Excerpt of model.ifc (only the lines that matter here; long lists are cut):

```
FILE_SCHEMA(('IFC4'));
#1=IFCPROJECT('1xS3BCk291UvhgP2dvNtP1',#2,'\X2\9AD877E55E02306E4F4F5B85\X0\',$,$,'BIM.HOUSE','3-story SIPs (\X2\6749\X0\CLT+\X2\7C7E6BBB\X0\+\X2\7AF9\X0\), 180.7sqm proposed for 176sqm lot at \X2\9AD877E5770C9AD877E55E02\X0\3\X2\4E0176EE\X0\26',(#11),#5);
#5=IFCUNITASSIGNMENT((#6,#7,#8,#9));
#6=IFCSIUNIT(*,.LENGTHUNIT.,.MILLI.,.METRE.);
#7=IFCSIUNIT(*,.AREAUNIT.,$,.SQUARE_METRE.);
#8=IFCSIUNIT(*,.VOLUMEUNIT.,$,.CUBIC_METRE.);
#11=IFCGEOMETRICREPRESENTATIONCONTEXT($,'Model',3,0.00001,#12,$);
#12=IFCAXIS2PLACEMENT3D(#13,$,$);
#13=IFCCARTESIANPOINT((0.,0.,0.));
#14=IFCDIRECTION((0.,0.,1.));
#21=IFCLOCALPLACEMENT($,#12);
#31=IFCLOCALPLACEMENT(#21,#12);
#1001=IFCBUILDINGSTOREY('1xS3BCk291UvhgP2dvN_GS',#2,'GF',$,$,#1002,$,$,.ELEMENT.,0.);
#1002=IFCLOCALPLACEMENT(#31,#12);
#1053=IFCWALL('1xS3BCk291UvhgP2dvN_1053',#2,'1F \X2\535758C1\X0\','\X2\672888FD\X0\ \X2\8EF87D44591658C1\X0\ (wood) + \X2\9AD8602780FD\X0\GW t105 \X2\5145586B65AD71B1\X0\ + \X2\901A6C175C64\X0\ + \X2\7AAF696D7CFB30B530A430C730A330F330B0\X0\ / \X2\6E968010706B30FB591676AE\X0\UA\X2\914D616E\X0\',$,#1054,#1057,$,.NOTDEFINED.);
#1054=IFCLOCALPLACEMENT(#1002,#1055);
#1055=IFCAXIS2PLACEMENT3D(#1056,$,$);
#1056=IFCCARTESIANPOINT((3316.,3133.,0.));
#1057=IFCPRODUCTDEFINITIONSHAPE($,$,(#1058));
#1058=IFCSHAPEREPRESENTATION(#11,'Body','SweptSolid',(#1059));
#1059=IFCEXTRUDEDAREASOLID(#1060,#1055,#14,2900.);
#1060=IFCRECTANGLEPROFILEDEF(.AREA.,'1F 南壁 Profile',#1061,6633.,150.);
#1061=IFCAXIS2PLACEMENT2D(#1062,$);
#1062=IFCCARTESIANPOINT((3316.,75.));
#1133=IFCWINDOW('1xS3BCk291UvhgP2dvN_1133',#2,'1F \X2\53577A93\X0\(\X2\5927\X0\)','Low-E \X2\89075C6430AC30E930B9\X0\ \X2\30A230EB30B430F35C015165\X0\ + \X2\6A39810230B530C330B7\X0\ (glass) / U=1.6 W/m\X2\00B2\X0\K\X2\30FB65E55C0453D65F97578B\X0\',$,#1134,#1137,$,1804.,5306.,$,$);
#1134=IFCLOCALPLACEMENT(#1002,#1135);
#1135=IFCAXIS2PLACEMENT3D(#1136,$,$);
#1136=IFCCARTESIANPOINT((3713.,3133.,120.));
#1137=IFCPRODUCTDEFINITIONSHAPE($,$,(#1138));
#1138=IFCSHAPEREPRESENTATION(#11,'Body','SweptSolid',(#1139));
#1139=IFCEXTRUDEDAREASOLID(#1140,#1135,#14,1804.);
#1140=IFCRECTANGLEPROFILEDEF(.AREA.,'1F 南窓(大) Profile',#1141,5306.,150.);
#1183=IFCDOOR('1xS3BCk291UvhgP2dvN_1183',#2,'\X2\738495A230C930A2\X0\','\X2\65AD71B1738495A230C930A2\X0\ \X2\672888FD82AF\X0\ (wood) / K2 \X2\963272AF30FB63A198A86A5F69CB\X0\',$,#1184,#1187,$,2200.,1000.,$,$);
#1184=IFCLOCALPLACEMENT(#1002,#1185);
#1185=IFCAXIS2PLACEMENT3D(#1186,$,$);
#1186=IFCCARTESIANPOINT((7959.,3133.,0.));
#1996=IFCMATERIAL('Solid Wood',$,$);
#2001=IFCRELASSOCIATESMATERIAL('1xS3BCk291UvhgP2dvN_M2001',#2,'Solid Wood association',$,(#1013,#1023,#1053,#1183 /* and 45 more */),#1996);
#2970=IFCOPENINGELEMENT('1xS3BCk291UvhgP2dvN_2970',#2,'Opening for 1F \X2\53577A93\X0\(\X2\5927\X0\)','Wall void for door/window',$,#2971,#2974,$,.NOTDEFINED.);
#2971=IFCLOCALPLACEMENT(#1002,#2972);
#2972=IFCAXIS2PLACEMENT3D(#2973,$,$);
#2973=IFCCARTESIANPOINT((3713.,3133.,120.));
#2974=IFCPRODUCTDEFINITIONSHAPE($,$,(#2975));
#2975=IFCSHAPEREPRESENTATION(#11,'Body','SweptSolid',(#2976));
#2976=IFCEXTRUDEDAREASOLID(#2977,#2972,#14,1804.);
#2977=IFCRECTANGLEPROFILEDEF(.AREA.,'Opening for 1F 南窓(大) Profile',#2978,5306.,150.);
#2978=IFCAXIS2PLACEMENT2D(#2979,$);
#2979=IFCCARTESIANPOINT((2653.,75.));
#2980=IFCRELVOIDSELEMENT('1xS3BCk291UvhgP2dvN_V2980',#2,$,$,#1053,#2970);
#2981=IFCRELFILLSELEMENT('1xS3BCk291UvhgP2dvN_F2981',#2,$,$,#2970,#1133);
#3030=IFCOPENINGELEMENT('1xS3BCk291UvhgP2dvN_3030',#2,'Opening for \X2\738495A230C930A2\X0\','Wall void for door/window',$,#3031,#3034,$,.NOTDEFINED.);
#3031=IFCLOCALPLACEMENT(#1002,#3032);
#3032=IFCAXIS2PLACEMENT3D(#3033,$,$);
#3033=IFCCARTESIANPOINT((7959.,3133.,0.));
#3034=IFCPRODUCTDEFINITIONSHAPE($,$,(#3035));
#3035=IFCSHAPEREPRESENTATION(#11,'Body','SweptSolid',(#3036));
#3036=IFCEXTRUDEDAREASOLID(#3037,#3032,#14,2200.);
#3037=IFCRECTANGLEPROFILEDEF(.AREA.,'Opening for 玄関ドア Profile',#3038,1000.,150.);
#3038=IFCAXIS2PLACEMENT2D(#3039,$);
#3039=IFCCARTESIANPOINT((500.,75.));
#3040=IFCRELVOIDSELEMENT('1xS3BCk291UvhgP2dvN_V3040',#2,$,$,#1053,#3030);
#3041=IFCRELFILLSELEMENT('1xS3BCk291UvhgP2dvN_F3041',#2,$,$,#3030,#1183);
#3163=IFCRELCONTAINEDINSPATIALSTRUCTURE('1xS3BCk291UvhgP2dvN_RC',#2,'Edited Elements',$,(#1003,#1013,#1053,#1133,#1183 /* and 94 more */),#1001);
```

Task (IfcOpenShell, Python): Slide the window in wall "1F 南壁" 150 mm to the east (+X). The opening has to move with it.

```python
import ifcopenshell
import ifcopenshell.api.geometry
import ifcopenshell.util.placement
import ifcopenshell.util.unit

model = ifcopenshell.open("model.ifc")
unit_scale = ifcopenshell.util.unit.calculate_unit_scale(model)

window = model.by_guid("1xS3BCk291UvhgP2dvN_1133")
opening = window.FillsVoids[0].RelatingOpeningElement
wall = opening.VoidsElements[0].RelatingBuildingElement

wall_matrix = ifcopenshell.util.placement.get_local_placement(wall.ObjectPlacement)
shift = wall_matrix[:3, 0] * 0.15 / unit_scale
before = ifcopenshell.util.placement.get_local_placement(window.ObjectPlacement)[:3, 3].copy()

# The window is not placed relative to its opening, so move both.
for product in (opening, window):
    matrix = ifcopenshell.util.placement.get_local_placement(product.ObjectPlacement)
    matrix[:3, 3] += shift
    ifcopenshell.api.geometry.edit_object_placement(model, product=product, matrix=matrix, is_si=False)

after = ifcopenshell.util.placement.get_local_placement(window.ObjectPlacement)[:3, 3]
print("window moved by", (after - before).round(3) + 0.0)

model.write("model_rev.ifc")
```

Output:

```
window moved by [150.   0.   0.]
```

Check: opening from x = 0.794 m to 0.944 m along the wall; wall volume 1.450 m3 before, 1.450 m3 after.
